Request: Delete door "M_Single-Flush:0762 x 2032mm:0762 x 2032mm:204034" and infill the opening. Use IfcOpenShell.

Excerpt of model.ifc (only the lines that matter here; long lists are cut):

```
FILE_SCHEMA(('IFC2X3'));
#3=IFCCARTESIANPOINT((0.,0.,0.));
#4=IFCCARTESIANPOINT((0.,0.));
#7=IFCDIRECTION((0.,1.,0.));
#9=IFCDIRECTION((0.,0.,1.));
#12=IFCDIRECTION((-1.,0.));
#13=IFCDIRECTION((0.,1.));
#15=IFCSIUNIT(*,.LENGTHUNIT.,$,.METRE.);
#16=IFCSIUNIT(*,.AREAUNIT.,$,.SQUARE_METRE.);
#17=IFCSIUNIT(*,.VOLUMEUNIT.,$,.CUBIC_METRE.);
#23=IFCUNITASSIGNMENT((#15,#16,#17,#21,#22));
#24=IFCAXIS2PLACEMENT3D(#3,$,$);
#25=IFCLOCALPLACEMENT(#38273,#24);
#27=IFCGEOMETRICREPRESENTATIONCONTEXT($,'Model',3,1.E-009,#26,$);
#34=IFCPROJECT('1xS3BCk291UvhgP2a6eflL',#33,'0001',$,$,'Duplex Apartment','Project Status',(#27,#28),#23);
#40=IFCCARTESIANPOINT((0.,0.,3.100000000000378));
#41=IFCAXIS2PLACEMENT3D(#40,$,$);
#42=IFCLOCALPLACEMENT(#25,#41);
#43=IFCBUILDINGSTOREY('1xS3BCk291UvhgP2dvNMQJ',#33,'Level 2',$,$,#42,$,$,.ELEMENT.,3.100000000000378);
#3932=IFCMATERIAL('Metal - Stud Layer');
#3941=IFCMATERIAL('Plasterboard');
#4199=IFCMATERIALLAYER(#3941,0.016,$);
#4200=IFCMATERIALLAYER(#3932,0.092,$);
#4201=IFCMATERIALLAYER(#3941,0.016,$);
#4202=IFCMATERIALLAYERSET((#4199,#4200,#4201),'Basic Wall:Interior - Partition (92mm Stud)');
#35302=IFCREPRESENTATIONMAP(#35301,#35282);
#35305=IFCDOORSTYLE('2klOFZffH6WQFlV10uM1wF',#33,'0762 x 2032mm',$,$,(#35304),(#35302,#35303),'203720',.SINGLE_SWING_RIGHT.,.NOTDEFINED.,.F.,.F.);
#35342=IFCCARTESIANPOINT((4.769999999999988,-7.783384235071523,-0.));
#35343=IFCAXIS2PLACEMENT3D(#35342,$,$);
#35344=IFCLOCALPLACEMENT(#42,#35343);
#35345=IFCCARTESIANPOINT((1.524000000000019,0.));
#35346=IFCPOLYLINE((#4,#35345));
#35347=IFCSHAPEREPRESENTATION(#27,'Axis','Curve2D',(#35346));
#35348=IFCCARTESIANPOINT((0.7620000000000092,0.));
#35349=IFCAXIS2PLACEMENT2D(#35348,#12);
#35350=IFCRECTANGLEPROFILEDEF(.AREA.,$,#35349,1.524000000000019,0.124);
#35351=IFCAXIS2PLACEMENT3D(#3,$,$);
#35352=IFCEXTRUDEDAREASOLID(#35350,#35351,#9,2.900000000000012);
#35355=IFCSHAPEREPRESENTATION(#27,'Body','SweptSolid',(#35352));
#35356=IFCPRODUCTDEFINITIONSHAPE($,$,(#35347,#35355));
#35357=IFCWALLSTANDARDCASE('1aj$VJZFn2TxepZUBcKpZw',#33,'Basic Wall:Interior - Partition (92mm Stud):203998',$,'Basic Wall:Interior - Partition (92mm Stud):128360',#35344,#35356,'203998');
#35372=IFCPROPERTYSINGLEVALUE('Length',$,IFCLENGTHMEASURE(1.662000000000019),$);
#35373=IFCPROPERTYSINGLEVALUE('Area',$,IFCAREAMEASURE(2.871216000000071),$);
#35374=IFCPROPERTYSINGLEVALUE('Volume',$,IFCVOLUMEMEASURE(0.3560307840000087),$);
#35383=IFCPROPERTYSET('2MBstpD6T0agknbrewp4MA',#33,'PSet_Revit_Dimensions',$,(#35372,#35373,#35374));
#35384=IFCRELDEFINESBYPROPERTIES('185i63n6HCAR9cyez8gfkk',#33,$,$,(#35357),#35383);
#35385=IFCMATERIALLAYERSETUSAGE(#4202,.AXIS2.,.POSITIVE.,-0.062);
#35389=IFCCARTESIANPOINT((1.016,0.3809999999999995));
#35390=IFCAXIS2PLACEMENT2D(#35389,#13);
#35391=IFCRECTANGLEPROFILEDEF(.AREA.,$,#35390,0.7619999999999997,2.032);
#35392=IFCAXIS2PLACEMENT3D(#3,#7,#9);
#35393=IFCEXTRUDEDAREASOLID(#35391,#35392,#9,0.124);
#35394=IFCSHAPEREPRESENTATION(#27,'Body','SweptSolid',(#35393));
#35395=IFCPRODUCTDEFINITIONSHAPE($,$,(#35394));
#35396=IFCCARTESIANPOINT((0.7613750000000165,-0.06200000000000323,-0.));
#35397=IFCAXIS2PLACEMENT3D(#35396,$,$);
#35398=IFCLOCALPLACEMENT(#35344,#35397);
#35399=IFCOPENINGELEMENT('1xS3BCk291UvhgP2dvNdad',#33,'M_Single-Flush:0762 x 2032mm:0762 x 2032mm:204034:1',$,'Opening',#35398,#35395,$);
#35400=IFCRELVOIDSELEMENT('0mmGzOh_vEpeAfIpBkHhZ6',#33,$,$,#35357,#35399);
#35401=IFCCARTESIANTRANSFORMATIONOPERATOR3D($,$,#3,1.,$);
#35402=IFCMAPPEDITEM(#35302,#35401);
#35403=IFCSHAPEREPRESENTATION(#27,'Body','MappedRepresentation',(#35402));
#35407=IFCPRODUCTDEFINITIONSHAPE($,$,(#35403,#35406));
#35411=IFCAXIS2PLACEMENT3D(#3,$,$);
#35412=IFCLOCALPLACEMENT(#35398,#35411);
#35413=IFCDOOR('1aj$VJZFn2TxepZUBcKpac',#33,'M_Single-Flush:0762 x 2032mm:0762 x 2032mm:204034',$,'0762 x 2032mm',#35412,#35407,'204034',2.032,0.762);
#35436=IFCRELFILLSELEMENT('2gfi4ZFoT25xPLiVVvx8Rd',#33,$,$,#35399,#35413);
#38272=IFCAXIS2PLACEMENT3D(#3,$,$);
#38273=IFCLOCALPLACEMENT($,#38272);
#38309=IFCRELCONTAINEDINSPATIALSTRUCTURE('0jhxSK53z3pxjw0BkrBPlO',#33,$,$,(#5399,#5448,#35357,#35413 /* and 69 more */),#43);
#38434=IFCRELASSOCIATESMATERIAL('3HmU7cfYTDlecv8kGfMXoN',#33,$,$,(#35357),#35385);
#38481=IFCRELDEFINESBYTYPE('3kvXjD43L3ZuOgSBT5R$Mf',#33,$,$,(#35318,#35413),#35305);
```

```python
import ifcopenshell
import ifcopenshell.api.feature
import ifcopenshell.api.pset
import ifcopenshell.api.root
import ifcopenshell.geom
import ifcopenshell.util.element
import ifcopenshell.util.shape
import ifcopenshell.util.unit

model = ifcopenshell.open("model.ifc")
area_scale = ifcopenshell.util.unit.calculate_unit_scale(model, "AREAUNIT")
volume_scale = ifcopenshell.util.unit.calculate_unit_scale(model, "VOLUMEUNIT")
settings = ifcopenshell.geom.settings()


def volume(element):
    """Net volume in cubic metres, openings subtracted."""
    shape = ifcopenshell.geom.create_shape(settings, element)
    return ifcopenshell.util.shape.get_volume(shape.geometry)


door = model.by_guid("1aj$VJZFn2TxepZUBcKpac")
opening = door.FillsVoids[0].RelatingOpeningElement
wall = opening.VoidsElements[0].RelatingBuildingElement
before = volume(wall)

ifcopenshell.api.root.remove_product(model, product=door)
ifcopenshell.api.feature.remove_feature(model, feature=opening)

after = volume(wall)
thickness = 0.124  # wall thickness in metres

# Update the wall's stored quantities.
pset = model.by_id(ifcopenshell.util.element.get_pset(wall, "PSet_Revit_Dimensions", should_inherit=False)["id"])
ifcopenshell.api.pset.edit_pset(model, pset=pset, properties={
    "Area": model.create_entity("IfcAreaMeasure", after / thickness / area_scale),
    "Volume": model.create_entity("IfcVolumeMeasure", after / volume_scale),
})

print(f"wall volume {before:.3f} -> {after:.3f} m3")

model.write("model_updated.ifc")
```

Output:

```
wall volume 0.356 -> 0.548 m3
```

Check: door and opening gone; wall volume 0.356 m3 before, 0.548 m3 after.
